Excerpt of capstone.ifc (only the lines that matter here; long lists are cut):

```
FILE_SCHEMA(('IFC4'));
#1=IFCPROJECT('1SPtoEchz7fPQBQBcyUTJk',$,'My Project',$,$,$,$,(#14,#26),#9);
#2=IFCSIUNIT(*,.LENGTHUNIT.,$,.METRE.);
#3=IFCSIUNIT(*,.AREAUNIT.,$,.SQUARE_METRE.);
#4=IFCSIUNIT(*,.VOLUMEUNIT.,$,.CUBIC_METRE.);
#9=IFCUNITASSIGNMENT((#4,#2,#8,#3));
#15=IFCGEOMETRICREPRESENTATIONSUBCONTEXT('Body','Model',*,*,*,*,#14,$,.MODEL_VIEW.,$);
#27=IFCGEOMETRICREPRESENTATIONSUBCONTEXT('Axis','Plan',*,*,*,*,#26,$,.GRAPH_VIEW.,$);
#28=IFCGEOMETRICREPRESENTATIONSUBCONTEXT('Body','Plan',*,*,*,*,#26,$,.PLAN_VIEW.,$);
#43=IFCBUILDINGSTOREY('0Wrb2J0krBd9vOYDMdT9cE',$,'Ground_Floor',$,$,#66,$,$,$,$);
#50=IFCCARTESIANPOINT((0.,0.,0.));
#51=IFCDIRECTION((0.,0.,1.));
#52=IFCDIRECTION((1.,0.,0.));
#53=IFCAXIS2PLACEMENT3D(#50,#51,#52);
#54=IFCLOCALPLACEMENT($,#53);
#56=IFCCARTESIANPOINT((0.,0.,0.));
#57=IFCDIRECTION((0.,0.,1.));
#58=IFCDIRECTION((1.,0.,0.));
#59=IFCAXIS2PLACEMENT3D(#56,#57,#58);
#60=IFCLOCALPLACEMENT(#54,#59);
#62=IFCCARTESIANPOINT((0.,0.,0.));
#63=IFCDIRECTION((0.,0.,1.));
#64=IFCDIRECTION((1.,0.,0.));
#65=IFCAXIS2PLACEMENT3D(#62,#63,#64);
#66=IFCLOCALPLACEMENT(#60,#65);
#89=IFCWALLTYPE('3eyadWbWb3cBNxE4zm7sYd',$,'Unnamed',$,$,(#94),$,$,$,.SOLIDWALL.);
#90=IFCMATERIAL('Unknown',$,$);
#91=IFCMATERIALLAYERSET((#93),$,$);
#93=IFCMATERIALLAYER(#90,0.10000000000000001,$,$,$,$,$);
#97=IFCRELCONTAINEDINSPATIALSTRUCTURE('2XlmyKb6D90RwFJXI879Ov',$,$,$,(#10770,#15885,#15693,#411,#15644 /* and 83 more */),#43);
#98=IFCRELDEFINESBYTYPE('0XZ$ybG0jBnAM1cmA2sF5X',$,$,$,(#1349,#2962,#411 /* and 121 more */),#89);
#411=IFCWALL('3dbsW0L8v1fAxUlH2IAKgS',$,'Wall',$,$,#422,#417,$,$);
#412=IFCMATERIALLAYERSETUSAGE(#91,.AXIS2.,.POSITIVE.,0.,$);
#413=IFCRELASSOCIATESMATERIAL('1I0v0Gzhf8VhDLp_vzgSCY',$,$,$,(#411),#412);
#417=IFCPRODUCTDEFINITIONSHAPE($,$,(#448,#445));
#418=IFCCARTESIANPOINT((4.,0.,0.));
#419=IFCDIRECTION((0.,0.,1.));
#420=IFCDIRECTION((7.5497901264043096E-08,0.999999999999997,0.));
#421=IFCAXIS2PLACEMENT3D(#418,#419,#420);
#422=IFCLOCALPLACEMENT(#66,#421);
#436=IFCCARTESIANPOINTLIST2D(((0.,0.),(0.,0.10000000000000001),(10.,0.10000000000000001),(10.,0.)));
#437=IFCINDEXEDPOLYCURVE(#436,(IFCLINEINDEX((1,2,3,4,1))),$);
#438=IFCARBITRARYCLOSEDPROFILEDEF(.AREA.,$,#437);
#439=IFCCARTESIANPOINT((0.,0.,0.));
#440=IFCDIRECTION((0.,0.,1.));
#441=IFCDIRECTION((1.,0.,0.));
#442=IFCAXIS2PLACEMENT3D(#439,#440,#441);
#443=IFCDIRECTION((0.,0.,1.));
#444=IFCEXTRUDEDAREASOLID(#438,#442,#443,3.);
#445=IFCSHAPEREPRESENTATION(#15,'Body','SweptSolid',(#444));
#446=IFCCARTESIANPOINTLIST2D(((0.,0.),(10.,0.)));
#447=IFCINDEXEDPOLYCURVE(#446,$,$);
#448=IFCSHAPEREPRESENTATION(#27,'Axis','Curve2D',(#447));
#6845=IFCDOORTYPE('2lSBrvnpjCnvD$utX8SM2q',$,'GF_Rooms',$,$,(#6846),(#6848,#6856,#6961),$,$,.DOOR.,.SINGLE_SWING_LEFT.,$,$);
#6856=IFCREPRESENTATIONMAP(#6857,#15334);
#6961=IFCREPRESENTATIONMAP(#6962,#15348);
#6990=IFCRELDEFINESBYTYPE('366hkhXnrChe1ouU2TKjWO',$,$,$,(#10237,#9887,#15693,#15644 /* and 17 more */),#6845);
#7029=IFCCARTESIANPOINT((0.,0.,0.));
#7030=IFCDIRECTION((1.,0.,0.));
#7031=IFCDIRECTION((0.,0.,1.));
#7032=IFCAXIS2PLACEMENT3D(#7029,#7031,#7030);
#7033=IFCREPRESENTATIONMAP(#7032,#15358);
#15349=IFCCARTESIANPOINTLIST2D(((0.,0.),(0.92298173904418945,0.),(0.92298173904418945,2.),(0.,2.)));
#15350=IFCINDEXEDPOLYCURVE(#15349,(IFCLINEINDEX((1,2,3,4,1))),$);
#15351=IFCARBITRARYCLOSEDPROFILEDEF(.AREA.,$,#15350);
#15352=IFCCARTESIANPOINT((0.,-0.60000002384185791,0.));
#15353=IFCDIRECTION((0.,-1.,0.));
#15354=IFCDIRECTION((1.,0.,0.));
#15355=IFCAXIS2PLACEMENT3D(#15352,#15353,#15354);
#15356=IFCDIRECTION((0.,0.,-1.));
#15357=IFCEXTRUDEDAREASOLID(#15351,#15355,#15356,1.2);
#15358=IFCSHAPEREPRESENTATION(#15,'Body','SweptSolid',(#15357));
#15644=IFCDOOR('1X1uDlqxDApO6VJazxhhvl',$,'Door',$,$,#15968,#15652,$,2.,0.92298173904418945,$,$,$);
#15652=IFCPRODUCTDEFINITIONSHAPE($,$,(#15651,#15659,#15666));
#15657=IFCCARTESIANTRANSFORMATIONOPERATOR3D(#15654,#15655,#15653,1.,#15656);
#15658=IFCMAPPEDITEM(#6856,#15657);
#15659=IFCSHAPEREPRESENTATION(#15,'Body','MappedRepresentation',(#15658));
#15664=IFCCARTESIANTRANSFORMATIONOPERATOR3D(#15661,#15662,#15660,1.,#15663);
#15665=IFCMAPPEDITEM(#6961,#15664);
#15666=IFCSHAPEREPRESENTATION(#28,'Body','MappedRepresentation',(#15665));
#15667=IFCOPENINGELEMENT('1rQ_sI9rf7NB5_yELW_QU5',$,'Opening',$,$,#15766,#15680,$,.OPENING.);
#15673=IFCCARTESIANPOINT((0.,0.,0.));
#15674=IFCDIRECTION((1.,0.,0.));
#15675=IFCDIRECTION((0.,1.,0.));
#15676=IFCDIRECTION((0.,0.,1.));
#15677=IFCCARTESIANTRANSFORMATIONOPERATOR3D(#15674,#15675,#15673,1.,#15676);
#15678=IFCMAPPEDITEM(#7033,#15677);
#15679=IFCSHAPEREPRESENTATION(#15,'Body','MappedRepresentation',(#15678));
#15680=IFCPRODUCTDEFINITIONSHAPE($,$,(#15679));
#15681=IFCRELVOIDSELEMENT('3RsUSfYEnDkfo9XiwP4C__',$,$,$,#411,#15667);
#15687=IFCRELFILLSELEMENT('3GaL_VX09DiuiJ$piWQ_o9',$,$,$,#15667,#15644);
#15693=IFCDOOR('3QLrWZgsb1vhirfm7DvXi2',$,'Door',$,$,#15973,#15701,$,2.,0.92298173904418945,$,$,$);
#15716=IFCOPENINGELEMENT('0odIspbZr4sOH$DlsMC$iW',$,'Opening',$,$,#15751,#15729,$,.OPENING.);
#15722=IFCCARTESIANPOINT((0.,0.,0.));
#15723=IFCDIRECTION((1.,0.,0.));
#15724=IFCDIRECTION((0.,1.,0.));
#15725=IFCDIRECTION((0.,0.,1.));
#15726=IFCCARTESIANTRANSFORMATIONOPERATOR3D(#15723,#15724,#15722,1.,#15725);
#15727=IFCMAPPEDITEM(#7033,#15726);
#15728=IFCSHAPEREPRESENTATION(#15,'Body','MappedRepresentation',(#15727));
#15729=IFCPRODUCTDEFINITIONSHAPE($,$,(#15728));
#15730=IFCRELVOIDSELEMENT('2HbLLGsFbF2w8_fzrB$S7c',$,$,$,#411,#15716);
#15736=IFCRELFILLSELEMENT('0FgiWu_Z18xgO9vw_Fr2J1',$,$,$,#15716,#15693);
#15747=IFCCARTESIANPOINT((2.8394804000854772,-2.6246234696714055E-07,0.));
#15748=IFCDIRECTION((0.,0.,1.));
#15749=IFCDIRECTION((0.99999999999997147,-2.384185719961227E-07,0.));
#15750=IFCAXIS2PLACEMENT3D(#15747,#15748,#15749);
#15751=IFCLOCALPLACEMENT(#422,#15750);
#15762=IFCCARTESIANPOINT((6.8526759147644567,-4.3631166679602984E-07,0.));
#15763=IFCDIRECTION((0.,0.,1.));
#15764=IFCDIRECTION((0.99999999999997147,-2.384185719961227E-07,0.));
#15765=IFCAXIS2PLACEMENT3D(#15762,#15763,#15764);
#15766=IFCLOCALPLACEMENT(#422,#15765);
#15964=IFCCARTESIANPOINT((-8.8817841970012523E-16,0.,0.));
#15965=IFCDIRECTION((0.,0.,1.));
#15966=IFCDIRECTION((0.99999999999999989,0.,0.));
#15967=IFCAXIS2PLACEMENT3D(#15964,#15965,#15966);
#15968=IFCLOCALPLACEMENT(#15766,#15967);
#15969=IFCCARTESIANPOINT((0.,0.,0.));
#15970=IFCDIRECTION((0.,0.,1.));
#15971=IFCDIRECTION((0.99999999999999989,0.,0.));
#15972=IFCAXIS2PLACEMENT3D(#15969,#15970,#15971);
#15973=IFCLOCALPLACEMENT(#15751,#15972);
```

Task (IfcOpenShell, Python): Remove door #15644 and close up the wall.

```python
import ifcopenshell
import ifcopenshell.api.feature
import ifcopenshell.api.root
import ifcopenshell.geom
import ifcopenshell.util.shape

model = ifcopenshell.open("capstone.ifc")
settings = ifcopenshell.geom.settings()


def volume(element):
    """Net volume in cubic metres, openings subtracted."""
    shape = ifcopenshell.geom.create_shape(settings, element)
    return ifcopenshell.util.shape.get_volume(shape.geometry)


door = model.by_guid("1X1uDlqxDApO6VJazxhhvl")
opening = door.FillsVoids[0].RelatingOpeningElement
wall = opening.VoidsElements[0].RelatingBuildingElement
before = volume(wall)

ifcopenshell.api.root.remove_product(model, product=door)
ifcopenshell.api.feature.remove_feature(model, feature=opening)

after = volume(wall)

print(f"wall volume {before:.3f} -> {after:.3f} m3")

model.write("capstone_updated.ifc")
```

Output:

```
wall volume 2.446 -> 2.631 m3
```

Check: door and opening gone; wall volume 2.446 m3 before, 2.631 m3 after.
